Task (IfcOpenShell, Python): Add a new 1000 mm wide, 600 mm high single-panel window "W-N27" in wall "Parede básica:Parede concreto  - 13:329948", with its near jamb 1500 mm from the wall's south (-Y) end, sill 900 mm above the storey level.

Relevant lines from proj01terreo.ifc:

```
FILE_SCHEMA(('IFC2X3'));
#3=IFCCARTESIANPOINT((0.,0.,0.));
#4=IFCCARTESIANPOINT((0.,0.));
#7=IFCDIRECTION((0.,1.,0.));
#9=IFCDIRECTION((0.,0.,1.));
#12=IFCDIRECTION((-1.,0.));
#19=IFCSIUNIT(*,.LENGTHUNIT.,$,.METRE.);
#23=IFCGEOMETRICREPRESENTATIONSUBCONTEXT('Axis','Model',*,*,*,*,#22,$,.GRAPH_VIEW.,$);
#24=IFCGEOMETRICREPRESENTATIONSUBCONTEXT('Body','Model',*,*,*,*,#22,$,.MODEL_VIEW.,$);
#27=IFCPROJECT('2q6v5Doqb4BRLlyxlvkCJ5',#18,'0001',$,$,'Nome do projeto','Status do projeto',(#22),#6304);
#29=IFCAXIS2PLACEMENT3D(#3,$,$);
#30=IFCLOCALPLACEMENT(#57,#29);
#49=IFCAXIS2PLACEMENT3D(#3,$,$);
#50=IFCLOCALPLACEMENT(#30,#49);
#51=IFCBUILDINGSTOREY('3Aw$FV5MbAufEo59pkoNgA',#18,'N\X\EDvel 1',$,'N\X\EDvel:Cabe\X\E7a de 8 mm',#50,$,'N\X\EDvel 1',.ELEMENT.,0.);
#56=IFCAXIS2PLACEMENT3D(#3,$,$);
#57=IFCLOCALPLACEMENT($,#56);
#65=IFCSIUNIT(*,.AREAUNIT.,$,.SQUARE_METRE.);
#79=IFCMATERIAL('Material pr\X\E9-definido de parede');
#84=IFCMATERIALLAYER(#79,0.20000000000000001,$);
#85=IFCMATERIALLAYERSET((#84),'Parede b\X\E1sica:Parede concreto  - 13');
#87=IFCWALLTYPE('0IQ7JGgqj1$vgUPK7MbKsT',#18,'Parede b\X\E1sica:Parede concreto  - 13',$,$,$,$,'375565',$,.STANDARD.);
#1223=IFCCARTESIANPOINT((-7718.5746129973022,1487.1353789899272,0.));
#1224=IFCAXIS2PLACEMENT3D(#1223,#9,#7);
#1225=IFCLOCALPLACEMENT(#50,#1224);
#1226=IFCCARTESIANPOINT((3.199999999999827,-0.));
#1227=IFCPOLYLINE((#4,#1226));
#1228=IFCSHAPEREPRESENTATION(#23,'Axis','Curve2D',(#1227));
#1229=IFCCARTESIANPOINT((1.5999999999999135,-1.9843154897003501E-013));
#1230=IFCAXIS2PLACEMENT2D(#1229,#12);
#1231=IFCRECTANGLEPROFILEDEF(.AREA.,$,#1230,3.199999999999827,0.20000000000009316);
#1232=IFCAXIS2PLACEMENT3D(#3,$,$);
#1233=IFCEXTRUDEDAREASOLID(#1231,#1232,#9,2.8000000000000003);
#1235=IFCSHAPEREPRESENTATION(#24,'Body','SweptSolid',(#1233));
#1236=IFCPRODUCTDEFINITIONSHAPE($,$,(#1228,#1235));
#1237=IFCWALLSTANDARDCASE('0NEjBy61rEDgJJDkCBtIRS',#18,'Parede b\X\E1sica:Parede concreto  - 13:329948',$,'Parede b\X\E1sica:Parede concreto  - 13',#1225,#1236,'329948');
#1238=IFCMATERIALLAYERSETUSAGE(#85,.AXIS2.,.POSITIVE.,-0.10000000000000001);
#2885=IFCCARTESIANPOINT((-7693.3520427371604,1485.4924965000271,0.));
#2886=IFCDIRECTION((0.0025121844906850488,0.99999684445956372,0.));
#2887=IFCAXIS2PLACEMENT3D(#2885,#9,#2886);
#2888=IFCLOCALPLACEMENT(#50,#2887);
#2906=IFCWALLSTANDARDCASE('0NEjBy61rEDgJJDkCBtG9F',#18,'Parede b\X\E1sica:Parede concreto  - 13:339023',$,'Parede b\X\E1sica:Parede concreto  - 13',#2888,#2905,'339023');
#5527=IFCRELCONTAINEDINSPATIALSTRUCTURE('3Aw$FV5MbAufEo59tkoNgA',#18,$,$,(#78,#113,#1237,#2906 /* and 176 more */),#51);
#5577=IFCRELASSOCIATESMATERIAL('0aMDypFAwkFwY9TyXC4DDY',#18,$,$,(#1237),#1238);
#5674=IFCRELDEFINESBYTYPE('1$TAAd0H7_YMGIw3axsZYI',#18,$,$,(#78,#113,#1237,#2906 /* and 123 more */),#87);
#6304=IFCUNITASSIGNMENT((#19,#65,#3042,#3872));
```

```python
import numpy as np
import ifcopenshell
import ifcopenshell.api.feature
import ifcopenshell.api.geometry
import ifcopenshell.api.root
import ifcopenshell.api.spatial
import ifcopenshell.api.type
import ifcopenshell.geom
import ifcopenshell.util.element
import ifcopenshell.util.placement
import ifcopenshell.util.representation
import ifcopenshell.util.shape
import ifcopenshell.util.unit

model = ifcopenshell.open("proj01terreo.ifc")
unit_scale = ifcopenshell.util.unit.calculate_unit_scale(model)
settings = ifcopenshell.geom.settings()


def volume(element):
    """Net volume in cubic metres, openings subtracted."""
    shape = ifcopenshell.geom.create_shape(settings, element)
    return ifcopenshell.util.shape.get_volume(shape.geometry)


wall = model.by_guid("0NEjBy61rEDgJJDkCBtIRS")
storey = ifcopenshell.util.element.get_container(wall, ifc_class="IfcBuildingStorey")
context = ifcopenshell.util.representation.get_context(model, "Model", "Body", "MODEL_VIEW")
before = volume(wall)

width, height, from_end, sill = 1, 0.6, 1.5, 0.9  # metres

# The wall runs along its own X axis, and the end named is its -X end.
wall_shape = ifcopenshell.geom.create_shape(settings, wall)
x, y, z = ifcopenshell.util.shape.get_vertices(wall_shape.geometry).T
start = x.min() + from_end
face, thickness = float(y.min()), float(y.max() - y.min())
wall_matrix = ifcopenshell.util.placement.get_local_placement(wall.ObjectPlacement)
level = ifcopenshell.util.placement.get_local_placement(storey.ObjectPlacement)[2, 3]


def in_wall(x, y):
    """Placement at x, y metres in the wall's axes, at sill height."""
    matrix = wall_matrix.copy()
    matrix[:, 3] = wall_matrix @ np.array([x / unit_scale, y / unit_scale, 0.0, 1.0])
    matrix[2, 3] = level + sill / unit_scale
    return matrix


# Opening: a box that overshoots both wall faces by 50 mm.
opening = ifcopenshell.api.root.create_entity(model, ifc_class="IfcOpeningElement")
box = ifcopenshell.api.geometry.add_wall_representation(
    model, context=context, length=width, height=height, thickness=thickness + 0.1
)
ifcopenshell.api.geometry.assign_representation(model, product=opening, representation=box)
ifcopenshell.api.geometry.edit_object_placement(model, product=opening, matrix=in_wall(start, face - 0.05), is_si=False)
ifcopenshell.api.feature.add_feature(model, feature=opening, element=wall)

window = ifcopenshell.api.root.create_entity(model, ifc_class="IfcWindow", name="W-N27")
window.OverallWidth, window.OverallHeight = width / unit_scale, height / unit_scale
body = ifcopenshell.api.geometry.add_window_representation(
    model,
    context=context,
    overall_width=window.OverallWidth,
    overall_height=window.OverallHeight,
    partition_type="SINGLE_PANEL",
)
ifcopenshell.api.geometry.assign_representation(model, product=window, representation=body)
ifcopenshell.api.spatial.assign_container(model, products=[window], relating_structure=storey)
fills = ifcopenshell.api.feature.add_filling(model, opening=opening, element=window)
fills.OwnerHistory = window.OwnerHistory  # required in IFC2X3

# IFC2X3 keeps the operation on the window style.
style = ifcopenshell.api.root.create_entity(model, ifc_class="IfcWindowStyle", name="W-N27")
style.OperationType, style.ConstructionType = "SINGLE_PANEL", "NOTDEFINED"
style.ParameterTakesPrecedence = style.Sizeable = False
ifcopenshell.api.type.assign_type(model, related_objects=[window], relating_type=style)

# Centre the window in the wall's thickness.
ifcopenshell.api.geometry.edit_object_placement(model, product=window, matrix=in_wall(start, face), is_si=False)
window_shape = ifcopenshell.geom.create_shape(settings, window)
depth = ifcopenshell.util.shape.get_vertices(window_shape.geometry)[:, 1]
offset = face + thickness / 2 - (depth.min() + depth.max()) / 2
ifcopenshell.api.geometry.edit_object_placement(model, product=window, matrix=in_wall(start, offset), is_si=False)

after = volume(wall)

print(f"wall volume {before:.3f} -> {after:.3f} m3")

model.write("proj01terreo_updated.ifc")
```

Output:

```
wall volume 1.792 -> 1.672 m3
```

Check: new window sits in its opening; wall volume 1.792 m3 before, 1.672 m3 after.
